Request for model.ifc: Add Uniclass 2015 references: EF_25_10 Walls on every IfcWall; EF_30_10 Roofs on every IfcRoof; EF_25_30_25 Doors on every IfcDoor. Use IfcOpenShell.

First a look at what the model holds.

```python
import ifcopenshell

model = ifcopenshell.open("model.ifc")
print(model.schema)
print("classifications:", [c.Name for c in model.by_type("IfcClassification")])
for ifc_class in ("IfcDoor", "IfcRoof", "IfcStair", "IfcWall", "IfcWindow"):
    print(ifc_class, len(model.by_type(ifc_class)))
```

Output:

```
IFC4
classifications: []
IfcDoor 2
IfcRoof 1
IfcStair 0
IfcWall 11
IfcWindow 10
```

```python
import ifcopenshell
import ifcopenshell.api.classification

model = ifcopenshell.open("model.ifc")

system = ifcopenshell.api.classification.add_classification(model, classification="Uniclass 2015")

codes = {
    "IfcWall": ("EF_25_10", "Walls"),
    "IfcRoof": ("EF_30_10", "Roofs"),
    "IfcDoor": ("EF_25_30_25", "Doors"),
}
for ifc_class, (code, name) in codes.items():
    products = model.by_type(ifc_class)
    ifcopenshell.api.classification.add_reference(
        model, products=products, classification=system, identification=code, name=name
    )
    print(code, len(products))

model.write("model-out.ifc")
```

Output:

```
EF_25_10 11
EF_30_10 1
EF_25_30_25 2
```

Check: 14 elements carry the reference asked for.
